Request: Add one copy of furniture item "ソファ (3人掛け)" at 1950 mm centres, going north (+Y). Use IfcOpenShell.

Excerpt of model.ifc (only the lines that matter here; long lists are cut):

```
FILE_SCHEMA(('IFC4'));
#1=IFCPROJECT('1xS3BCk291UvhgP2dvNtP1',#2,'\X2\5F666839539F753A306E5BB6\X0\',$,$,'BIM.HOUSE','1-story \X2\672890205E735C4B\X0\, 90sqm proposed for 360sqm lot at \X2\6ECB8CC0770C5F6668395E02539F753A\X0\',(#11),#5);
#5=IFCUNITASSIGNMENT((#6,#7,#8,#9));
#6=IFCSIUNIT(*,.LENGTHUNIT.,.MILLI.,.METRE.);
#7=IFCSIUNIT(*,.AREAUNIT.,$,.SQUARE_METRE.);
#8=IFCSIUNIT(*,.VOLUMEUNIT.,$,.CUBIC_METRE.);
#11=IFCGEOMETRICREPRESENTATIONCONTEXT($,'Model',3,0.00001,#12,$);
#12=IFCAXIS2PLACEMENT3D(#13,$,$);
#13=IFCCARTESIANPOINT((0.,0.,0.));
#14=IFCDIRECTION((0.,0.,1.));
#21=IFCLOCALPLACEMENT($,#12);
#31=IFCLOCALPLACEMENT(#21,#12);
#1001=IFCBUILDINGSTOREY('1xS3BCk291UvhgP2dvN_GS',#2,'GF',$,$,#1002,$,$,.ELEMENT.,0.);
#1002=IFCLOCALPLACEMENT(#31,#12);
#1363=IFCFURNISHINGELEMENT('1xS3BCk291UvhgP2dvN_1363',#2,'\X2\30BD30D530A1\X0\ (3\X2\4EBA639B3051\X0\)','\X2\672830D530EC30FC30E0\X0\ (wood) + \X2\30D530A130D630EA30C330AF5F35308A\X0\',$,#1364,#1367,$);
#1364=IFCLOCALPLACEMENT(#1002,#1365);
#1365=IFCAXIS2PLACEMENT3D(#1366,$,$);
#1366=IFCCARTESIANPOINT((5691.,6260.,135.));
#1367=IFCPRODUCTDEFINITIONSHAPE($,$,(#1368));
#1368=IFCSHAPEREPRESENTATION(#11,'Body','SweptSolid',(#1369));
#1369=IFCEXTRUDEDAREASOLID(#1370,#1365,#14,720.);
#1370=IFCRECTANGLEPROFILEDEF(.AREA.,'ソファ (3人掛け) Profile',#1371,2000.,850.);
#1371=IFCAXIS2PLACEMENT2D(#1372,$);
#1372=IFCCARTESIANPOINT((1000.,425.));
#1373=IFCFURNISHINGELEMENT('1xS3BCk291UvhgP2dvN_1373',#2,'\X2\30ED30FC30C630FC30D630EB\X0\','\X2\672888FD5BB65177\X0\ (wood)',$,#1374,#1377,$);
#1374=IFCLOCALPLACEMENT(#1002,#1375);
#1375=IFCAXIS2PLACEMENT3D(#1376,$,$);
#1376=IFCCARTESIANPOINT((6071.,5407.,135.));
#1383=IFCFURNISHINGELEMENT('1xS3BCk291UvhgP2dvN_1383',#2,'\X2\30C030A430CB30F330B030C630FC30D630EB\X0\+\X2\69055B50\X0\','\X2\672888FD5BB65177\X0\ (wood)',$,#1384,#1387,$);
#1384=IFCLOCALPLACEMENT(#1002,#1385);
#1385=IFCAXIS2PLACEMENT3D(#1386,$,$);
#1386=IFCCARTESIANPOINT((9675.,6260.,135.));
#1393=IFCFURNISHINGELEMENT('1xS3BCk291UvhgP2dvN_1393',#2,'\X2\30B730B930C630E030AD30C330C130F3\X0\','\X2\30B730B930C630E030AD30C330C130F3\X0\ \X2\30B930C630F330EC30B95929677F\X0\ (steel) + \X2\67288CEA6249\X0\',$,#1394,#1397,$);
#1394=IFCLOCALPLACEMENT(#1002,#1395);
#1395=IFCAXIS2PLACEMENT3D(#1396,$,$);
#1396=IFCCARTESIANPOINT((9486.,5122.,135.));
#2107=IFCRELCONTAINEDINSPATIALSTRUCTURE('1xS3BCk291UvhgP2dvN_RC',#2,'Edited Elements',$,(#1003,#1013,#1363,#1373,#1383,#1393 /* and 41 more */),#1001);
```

```python
import numpy as np
import ifcopenshell
import ifcopenshell.api.geometry
import ifcopenshell.api.root
import ifcopenshell.util.element
import ifcopenshell.util.placement
import ifcopenshell.util.unit

model = ifcopenshell.open("model.ifc")
unit_scale = ifcopenshell.util.unit.calculate_unit_scale(model)


def reuse_history(source, copy):
    """copy_class also copies each property set's owner history, people and application; keep the originals."""
    for rel in copy.IsDefinedBy:
        if rel.is_a("IfcRelDefinesByProperties") and (history := rel.RelatingPropertyDefinition.OwnerHistory):
            rel.RelatingPropertyDefinition.OwnerHistory = source.OwnerHistory
            ifcopenshell.util.element.remove_deep2(model, history)


source = model.by_guid("1xS3BCk291UvhgP2dvN_1363")
base = ifcopenshell.util.placement.get_local_placement(source.ObjectPlacement)
step = np.array([0.0, 1.0, 0.0]) * 1.95 / unit_scale

for i in range(1, 2):
    copy = ifcopenshell.api.root.copy_class(model, product=source)
    copy.Representation = ifcopenshell.util.element.copy_deep(
        model, source.Representation, exclude=["IfcGeometricRepresentationContext", "IfcRepresentationMap"]
    )
    reuse_history(source, copy)
    matrix = base.copy()
    matrix[:3, 3] += i * step
    print("added at", matrix[:3, 3].round(3) + 0.0)
    ifcopenshell.api.geometry.edit_object_placement(model, product=copy, matrix=matrix, is_si=False)

model.write("model_v2.ifc")
```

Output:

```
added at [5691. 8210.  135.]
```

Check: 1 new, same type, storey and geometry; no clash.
